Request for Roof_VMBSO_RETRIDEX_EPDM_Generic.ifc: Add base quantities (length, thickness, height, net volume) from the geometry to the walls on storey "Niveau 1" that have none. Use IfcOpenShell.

First a look at what the model holds.

```python
import ifcopenshell
import ifcopenshell.util.element
import ifcopenshell.util.unit

model = ifcopenshell.open("Roof_VMBSO_RETRIDEX_EPDM_Generic.ifc")
print(model.schema)
for unit_type in ("LENGTHUNIT", "AREAUNIT", "VOLUMEUNIT"):
    print(unit_type, ifcopenshell.util.unit.calculate_unit_scale(model, unit_type))
storey = next(s for s in model.by_type("IfcBuildingStorey") if s.Name == "Niveau 1")
walls = [e for e in ifcopenshell.util.element.get_decomposition(storey) if e.is_a("IfcWall")]
for e in sorted(walls, key=lambda e: e.id()):
    print(e.id(), e.is_a(), e.Name, list(ifcopenshell.util.element.get_psets(e, qtos_only=True)), sep=" | ")
```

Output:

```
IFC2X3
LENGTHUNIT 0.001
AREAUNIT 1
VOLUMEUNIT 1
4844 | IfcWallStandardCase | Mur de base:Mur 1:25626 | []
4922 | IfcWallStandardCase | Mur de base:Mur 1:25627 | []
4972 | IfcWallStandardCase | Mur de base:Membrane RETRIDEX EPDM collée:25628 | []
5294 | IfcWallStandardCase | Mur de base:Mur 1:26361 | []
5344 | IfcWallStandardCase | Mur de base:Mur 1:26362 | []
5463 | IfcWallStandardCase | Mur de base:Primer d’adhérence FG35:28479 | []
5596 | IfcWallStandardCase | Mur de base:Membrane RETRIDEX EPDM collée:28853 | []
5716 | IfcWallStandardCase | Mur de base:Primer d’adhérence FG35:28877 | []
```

```python
import ifcopenshell
import ifcopenshell.api.pset
import ifcopenshell.geom
import ifcopenshell.util.element
import ifcopenshell.util.shape
import ifcopenshell.util.unit

model = ifcopenshell.open("Roof_VMBSO_RETRIDEX_EPDM_Generic.ifc")
unit_scale = ifcopenshell.util.unit.calculate_unit_scale(model)
volume_scale = ifcopenshell.util.unit.calculate_unit_scale(model, "VOLUMEUNIT")
settings = ifcopenshell.geom.settings()

storey = next(s for s in model.by_type("IfcBuildingStorey") if s.Name == "Niveau 1")
walls = [e for e in ifcopenshell.util.element.get_decomposition(storey) if e.is_a("IfcWall")]

for e in sorted(walls, key=lambda e: e.id()):
    if ifcopenshell.util.element.get_psets(e, qtos_only=True, should_inherit=False):
        continue
    # Geometry comes back in metres, in the element's own axes.
    shape = ifcopenshell.geom.create_shape(settings, e)
    values = {
        "Length": ifcopenshell.util.shape.get_x(shape.geometry) / unit_scale,
        "Width": ifcopenshell.util.shape.get_y(shape.geometry) / unit_scale,
        "Height": ifcopenshell.util.shape.get_z(shape.geometry) / unit_scale,
        "NetVolume": ifcopenshell.util.shape.get_volume(shape.geometry) / volume_scale,
    }
    qto = ifcopenshell.api.pset.add_qto(model, product=e, name="BaseQuantities")
    ifcopenshell.api.pset.edit_qto(model, qto=qto, properties=values)
    print(e.id(), {k: round(v, 3) for k, v in values.items()})

model.write("Roof_VMBSO_RETRIDEX_EPDM_Generic_updated.ifc")
```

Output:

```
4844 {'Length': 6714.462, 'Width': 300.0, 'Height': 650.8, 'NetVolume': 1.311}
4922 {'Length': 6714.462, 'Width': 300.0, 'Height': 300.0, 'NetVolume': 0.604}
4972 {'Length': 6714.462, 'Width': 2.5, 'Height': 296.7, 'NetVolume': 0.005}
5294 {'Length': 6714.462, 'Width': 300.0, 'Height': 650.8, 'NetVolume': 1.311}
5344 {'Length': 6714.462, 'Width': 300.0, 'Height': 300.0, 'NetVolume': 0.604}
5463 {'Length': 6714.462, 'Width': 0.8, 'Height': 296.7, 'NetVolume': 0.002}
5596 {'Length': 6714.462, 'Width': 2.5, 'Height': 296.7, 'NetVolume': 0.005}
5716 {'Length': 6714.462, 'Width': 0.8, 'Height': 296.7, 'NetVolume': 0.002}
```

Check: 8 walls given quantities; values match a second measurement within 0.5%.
